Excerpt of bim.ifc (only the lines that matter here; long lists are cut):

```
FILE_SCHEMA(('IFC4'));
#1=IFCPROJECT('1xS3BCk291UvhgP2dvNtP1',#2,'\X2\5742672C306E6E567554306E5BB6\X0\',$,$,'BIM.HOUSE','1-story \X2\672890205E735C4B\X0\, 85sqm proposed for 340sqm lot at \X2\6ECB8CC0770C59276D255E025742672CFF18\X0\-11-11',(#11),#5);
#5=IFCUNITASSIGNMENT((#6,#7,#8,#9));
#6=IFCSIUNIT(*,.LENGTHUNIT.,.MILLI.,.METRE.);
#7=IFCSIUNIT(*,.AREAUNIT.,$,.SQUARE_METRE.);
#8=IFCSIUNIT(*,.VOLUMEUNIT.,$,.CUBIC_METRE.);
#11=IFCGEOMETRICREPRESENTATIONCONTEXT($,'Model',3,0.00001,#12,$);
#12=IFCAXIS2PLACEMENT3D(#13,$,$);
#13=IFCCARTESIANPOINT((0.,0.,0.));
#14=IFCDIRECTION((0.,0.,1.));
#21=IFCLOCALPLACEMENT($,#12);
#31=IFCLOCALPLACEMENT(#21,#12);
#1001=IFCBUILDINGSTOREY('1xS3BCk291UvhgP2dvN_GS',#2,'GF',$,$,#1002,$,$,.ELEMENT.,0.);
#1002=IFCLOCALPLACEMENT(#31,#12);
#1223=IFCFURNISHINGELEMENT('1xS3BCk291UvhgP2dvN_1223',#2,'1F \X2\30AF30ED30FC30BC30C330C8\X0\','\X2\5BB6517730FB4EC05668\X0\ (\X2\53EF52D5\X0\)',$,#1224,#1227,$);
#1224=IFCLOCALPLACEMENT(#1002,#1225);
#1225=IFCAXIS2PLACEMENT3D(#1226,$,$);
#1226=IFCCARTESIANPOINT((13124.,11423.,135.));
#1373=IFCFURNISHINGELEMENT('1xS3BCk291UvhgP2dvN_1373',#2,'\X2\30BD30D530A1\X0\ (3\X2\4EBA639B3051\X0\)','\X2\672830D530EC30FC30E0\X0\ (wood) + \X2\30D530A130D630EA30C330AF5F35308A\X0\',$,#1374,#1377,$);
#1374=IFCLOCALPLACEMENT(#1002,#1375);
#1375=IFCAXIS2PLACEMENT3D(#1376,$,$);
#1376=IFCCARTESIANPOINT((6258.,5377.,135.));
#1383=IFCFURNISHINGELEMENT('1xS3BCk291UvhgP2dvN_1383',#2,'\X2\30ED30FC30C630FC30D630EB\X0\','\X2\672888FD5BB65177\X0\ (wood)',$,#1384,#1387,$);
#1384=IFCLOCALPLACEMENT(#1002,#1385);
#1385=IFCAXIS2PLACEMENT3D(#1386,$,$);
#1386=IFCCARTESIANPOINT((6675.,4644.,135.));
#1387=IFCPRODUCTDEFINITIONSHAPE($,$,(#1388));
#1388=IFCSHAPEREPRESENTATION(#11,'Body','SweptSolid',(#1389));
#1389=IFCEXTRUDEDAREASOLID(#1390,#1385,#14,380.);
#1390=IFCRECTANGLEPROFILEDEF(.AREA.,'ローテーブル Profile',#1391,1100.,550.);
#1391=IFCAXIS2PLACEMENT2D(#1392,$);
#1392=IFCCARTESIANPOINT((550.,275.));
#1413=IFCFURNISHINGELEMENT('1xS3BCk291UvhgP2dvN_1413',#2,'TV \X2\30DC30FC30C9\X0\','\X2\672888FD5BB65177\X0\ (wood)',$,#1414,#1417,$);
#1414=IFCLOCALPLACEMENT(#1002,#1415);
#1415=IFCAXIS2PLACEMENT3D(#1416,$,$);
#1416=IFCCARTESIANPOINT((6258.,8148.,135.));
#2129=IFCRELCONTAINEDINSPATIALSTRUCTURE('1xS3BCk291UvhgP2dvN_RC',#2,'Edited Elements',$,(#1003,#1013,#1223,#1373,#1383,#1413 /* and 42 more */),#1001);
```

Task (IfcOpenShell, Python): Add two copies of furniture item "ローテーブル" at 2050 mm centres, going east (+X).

```python
import numpy as np
import ifcopenshell
import ifcopenshell.api.geometry
import ifcopenshell.api.root
import ifcopenshell.util.element
import ifcopenshell.util.placement

model = ifcopenshell.open("bim.ifc")


def reuse_history(source, copy):
    """copy_class also copies each property set's owner history, people and application; keep the originals."""
    for rel in copy.IsDefinedBy:
        if rel.is_a("IfcRelDefinesByProperties") and (history := rel.RelatingPropertyDefinition.OwnerHistory):
            rel.RelatingPropertyDefinition.OwnerHistory = source.OwnerHistory
            ifcopenshell.util.element.remove_deep2(model, history)


source = model.by_id(1383)
base = ifcopenshell.util.placement.get_local_placement(source.ObjectPlacement)
step = np.array([1.0, 0.0, 0.0]) * 2050.0

for i in range(1, 3):
    copy = ifcopenshell.api.root.copy_class(model, product=source)
    copy.Representation = ifcopenshell.util.element.copy_deep(
        model, source.Representation, exclude=["IfcGeometricRepresentationContext", "IfcRepresentationMap"]
    )
    reuse_history(source, copy)
    matrix = base.copy()
    matrix[:3, 3] += i * step
    print("added at", matrix[:3, 3].round(3) + 0.0)
    ifcopenshell.api.geometry.edit_object_placement(model, product=copy, matrix=matrix, is_si=False)

model.write("bim_edited.ifc")
```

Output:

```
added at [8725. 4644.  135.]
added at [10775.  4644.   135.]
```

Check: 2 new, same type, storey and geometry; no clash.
